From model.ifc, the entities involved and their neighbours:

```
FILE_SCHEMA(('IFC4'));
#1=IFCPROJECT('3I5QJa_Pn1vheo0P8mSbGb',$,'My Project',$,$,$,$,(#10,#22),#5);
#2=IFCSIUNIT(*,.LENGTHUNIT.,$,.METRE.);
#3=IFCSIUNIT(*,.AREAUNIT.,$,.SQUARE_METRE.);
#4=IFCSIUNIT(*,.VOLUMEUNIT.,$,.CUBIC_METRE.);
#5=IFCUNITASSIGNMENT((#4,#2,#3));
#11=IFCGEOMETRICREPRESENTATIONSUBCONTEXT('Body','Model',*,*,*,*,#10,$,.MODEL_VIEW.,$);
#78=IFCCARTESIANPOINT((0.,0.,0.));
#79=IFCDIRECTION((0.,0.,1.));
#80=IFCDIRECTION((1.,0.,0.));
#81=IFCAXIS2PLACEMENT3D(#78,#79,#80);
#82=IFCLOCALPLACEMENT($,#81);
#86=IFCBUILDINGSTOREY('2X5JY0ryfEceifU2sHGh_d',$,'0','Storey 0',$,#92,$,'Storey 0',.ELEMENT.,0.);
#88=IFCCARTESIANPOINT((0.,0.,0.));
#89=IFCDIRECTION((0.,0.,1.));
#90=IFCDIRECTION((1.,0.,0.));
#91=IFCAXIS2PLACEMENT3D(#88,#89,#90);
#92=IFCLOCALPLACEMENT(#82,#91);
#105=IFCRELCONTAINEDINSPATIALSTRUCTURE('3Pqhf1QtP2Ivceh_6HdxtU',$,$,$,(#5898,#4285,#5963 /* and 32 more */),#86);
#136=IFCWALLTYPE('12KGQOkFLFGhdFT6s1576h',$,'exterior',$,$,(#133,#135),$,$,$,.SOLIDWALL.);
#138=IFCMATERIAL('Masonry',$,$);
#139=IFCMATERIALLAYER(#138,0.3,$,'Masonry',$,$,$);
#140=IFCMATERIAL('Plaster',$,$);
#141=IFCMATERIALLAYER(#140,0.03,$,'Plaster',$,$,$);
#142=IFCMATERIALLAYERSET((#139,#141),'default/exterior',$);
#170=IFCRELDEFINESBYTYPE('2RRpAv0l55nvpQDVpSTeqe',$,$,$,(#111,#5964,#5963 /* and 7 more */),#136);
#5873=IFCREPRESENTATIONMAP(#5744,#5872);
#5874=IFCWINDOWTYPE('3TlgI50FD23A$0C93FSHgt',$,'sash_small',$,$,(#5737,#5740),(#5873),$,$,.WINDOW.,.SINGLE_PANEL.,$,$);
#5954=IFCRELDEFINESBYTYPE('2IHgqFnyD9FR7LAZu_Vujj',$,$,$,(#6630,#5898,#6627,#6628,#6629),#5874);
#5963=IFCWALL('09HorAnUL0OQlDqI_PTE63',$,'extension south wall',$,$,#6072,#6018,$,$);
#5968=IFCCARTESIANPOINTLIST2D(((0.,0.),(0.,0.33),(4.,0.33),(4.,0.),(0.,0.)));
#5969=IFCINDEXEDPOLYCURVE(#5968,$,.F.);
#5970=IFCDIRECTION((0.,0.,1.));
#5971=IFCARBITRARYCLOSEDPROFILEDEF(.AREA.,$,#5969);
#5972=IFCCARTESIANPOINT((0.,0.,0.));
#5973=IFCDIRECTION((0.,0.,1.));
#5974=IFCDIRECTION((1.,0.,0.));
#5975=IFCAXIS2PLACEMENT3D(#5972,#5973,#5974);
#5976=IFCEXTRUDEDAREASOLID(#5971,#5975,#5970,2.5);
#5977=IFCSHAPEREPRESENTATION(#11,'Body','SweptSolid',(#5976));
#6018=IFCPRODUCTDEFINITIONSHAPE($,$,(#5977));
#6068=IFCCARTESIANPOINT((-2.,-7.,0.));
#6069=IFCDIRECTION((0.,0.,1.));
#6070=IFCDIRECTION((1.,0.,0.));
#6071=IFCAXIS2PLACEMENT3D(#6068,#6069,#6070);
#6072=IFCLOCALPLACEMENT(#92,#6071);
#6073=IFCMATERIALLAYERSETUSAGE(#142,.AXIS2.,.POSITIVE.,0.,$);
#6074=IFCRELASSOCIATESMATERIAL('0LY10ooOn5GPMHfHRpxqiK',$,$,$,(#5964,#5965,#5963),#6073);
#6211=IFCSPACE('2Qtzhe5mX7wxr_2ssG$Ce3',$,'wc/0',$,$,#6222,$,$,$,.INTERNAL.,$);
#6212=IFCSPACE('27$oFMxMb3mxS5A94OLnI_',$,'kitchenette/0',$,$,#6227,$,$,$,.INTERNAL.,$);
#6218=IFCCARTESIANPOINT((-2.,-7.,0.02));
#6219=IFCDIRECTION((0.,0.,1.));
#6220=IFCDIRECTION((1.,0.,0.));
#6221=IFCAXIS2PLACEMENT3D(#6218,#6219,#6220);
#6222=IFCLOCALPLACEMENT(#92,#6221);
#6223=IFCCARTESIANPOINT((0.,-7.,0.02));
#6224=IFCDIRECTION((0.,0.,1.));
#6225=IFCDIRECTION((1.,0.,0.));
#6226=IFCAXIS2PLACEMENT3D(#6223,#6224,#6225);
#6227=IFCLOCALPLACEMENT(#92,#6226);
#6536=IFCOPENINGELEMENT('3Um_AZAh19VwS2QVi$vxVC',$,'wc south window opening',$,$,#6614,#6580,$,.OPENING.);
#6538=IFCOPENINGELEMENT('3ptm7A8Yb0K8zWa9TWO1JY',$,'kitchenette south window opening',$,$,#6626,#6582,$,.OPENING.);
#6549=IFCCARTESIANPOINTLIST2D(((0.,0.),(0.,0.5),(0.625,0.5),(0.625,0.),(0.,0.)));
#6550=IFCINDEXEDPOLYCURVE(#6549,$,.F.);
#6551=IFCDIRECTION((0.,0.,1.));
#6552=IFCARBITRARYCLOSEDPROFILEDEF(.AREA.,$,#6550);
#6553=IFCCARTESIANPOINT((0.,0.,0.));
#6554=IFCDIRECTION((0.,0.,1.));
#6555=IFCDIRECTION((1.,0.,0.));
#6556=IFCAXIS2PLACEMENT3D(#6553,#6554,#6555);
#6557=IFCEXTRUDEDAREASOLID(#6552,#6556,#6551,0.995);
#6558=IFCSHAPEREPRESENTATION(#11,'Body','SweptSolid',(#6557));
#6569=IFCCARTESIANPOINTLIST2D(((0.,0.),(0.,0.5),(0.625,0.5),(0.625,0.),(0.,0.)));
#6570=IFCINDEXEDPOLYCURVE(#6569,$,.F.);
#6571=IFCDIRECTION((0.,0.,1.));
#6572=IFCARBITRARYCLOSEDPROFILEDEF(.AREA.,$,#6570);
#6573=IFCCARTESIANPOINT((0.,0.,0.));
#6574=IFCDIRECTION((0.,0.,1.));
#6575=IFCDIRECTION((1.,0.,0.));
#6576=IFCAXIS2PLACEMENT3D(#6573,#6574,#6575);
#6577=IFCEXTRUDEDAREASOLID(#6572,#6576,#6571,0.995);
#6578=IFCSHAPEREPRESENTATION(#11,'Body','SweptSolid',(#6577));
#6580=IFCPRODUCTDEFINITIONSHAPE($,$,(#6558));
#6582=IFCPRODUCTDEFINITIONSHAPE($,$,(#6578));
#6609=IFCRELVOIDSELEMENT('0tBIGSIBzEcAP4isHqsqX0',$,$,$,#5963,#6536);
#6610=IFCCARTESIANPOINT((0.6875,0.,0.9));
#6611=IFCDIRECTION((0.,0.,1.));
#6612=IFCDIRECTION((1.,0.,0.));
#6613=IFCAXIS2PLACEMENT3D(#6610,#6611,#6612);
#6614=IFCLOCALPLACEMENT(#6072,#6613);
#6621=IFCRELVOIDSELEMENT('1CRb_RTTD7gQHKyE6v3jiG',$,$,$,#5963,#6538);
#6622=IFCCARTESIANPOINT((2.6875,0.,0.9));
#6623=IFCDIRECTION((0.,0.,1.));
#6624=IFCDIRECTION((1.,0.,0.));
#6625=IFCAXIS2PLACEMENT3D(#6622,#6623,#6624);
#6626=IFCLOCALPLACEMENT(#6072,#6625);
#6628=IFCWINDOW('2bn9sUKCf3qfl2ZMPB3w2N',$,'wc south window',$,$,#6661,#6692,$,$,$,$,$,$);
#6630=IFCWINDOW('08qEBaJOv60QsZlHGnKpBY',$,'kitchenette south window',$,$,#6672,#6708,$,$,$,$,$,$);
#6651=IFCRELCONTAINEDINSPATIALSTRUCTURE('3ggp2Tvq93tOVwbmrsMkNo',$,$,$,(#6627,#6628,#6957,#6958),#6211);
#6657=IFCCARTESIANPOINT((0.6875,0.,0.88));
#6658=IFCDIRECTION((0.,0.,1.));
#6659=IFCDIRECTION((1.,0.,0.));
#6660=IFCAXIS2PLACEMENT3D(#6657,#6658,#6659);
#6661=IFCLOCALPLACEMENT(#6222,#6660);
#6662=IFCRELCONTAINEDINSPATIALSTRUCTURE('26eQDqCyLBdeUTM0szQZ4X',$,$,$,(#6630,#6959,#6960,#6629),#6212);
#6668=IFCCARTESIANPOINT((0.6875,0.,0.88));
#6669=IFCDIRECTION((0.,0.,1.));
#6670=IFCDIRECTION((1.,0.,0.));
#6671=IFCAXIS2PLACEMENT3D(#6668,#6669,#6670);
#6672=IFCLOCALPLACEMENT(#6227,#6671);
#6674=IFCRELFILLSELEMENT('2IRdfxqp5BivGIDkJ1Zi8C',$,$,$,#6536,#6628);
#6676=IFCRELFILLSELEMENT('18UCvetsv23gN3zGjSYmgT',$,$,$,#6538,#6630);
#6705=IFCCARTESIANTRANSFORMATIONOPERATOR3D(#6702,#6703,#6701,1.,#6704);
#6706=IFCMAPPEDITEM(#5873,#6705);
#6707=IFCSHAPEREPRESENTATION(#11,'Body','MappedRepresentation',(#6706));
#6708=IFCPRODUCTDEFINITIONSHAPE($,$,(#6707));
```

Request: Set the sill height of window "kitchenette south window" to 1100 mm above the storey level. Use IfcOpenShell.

```python
import numpy as np
import ifcopenshell
import ifcopenshell.api.geometry
import ifcopenshell.geom
import ifcopenshell.util.element
import ifcopenshell.util.placement
import ifcopenshell.util.shape
import ifcopenshell.util.unit

model = ifcopenshell.open("model.ifc")
unit_scale = ifcopenshell.util.unit.calculate_unit_scale(model)

window = model.by_guid("08qEBaJOv60QsZlHGnKpBY")
opening = window.FillsVoids[0].RelatingOpeningElement
storey = ifcopenshell.util.element.get_container(window, ifc_class="IfcBuildingStorey")
level = ifcopenshell.util.placement.get_local_placement(storey.ObjectPlacement)[2, 3]

# The opening's origin need not be at the sill, so measure its lowest point.
shape = ifcopenshell.geom.create_shape(ifcopenshell.geom.settings(), opening)
bottom = ifcopenshell.util.shape.get_shape_bottom_elevation(shape, shape.geometry) / unit_scale
dz = level + 1.1 - bottom

shift = np.array([0.0, 0.0, dz])
# The window is not placed relative to its opening, so move both.
for product in (opening, window):
    matrix = ifcopenshell.util.placement.get_local_placement(product.ObjectPlacement)
    matrix[:3, 3] += shift
    ifcopenshell.api.geometry.edit_object_placement(model, product=product, matrix=matrix, is_si=False)

print(f"moved by {dz * unit_scale:+.3f} m")

model.write("model_rev.ifc")
```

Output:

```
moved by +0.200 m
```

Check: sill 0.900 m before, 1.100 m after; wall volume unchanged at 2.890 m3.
